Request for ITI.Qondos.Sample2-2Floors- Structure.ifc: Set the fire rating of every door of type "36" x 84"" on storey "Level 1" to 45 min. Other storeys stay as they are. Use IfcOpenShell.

First a look at what the model holds.

```python
import ifcopenshell
import ifcopenshell.util.element

model = ifcopenshell.open("ITI.Qondos.Sample2-2Floors- Structure.ifc")
print(model.schema)
storey = next(s for s in model.by_type("IfcBuildingStorey") if s.Name == "Level 1")
doors = [e for e in ifcopenshell.util.element.get_decomposition(storey) if e.is_a("IfcDoor")]
seen = {}
for e in doors:
    element_type = ifcopenshell.util.element.get_type(e)
    key = (element_type.Name if element_type != e and element_type else None, ifcopenshell.util.element.get_pset(e, "Pset_DoorCommon", "FireRating"))
    seen[key] = seen.get(key, 0) + 1
for (name, value), count in sorted(seen.items(), key=str):
    print(count, "x", name, "|", value)
```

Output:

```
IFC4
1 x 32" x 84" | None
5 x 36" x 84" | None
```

```python
import ifcopenshell
import ifcopenshell.api.pset
import ifcopenshell.util.element

model = ifcopenshell.open("ITI.Qondos.Sample2-2Floors- Structure.ifc")

storey = next(s for s in model.by_type("IfcBuildingStorey") if s.Name == "Level 1")
doors = [e for e in ifcopenshell.util.element.get_decomposition(storey) if e.is_a("IfcDoor")]

count = 0
for e in doors:
    element_type = ifcopenshell.util.element.get_type(e)
    if element_type in (None, e) or element_type.Name != '36" x 84"':
        continue
    # add_pset returns the element's existing set when there is one.
    pset = ifcopenshell.api.pset.add_pset(model, product=e, name="Pset_DoorCommon")
    ifcopenshell.api.pset.edit_pset(model, pset=pset, properties={"FireRating": "45 min"})
    count += 1

print(count, "doors updated")

model.write("ITI.Qondos.Sample2-2Floors- Structure_rev.ifc")
```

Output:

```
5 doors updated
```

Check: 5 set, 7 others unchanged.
